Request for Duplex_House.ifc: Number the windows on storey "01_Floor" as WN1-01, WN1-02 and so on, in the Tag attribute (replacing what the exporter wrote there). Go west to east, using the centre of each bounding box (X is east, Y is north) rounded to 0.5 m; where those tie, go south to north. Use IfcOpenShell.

First a look at what the model holds.

```python
import ifcopenshell
import ifcopenshell.util.element
import ifcopenshell.util.placement

model = ifcopenshell.open("Duplex_House.ifc")
print(model.schema)
storey = next(s for s in model.by_type("IfcBuildingStorey") if s.Name == "01_Floor")
windows = [e for e in ifcopenshell.util.element.get_decomposition(storey) if e.is_a("IfcWindow")]
for e in sorted(windows, key=lambda e: e.id()):
    origin = ifcopenshell.util.placement.get_local_placement(e.ObjectPlacement)[:3, 3]
    print(e.id(), e.Tag, e.Name, origin.round(2) + 0.0, sep=" | ")
```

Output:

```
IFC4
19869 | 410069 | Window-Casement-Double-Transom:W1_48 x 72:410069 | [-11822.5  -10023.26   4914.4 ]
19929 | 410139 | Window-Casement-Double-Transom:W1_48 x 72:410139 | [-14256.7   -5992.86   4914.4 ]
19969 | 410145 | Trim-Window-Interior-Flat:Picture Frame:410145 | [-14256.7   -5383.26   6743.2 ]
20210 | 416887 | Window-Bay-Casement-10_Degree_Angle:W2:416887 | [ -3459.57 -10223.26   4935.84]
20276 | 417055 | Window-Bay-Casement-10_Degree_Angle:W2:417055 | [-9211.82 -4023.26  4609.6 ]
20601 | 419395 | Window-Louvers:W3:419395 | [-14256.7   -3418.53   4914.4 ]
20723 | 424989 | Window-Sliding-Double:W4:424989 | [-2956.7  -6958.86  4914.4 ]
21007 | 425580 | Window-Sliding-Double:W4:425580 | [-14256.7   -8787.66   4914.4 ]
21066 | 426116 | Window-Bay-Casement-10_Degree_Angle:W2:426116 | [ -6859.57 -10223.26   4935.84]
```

```python
import ifcopenshell
import ifcopenshell.geom
import ifcopenshell.util.element
import ifcopenshell.util.shape

model = ifcopenshell.open("Duplex_House.ifc")
settings = ifcopenshell.geom.settings()
settings.set("use-world-coords", True)


def centre(element):
    shape = ifcopenshell.geom.create_shape(settings, element)
    return ifcopenshell.util.shape.get_bbox_centroid(shape.geometry)


storey = next(s for s in model.by_type("IfcBuildingStorey") if s.Name == "01_Floor")
windows = [e for e in ifcopenshell.util.element.get_decomposition(storey) if e.is_a("IfcWindow")]

# Insertion points can sit at a corner or the storey origin, so sort by the geometry (in metres).
centres = {e: centre(e) for e in windows}
windows.sort(key=lambda e: (round(centres[e][0] / 0.5), centres[e][1]))

for i, e in enumerate(windows, start=1):
    number = f"WN1-{i:02d}"
    e.Tag = number
    print(e.id(), number)

model.write("Duplex_House_rev.ifc")
```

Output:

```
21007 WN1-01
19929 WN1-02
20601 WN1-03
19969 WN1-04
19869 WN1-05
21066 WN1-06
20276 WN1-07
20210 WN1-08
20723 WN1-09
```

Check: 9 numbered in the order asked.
